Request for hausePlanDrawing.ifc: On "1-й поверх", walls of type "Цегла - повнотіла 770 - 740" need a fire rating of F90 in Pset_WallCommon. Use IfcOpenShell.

First a look at what the model holds.

```python
import ifcopenshell
import ifcopenshell.util.element

model = ifcopenshell.open("hausePlanDrawing.ifc")
print(model.schema)
storey = next(s for s in model.by_type("IfcBuildingStorey") if s.Name == "1-й поверх")
walls = [e for e in ifcopenshell.util.element.get_decomposition(storey) if e.is_a("IfcWall")]
seen = {}
for e in walls:
    element_type = ifcopenshell.util.element.get_type(e)
    key = (element_type.Name if element_type != e and element_type else None, ifcopenshell.util.element.get_pset(e, "Pset_WallCommon", "FireRating"))
    seen[key] = seen.get(key, 0) + 1
for (name, value), count in sorted(seen.items(), key=str):
    print(count, "x", name, "|", value)
```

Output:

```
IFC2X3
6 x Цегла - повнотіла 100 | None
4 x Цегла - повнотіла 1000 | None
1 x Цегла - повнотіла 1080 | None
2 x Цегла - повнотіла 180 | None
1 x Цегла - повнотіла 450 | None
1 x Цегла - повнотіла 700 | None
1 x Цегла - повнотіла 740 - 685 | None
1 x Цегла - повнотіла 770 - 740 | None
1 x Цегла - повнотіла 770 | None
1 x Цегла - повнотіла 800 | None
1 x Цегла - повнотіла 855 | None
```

```python
import ifcopenshell
import ifcopenshell.api.pset
import ifcopenshell.util.element

model = ifcopenshell.open("hausePlanDrawing.ifc")

storey = next(s for s in model.by_type("IfcBuildingStorey") if s.Name == "1-й поверх")
walls = [e for e in ifcopenshell.util.element.get_decomposition(storey) if e.is_a("IfcWall")]

count = 0
for e in walls:
    element_type = ifcopenshell.util.element.get_type(e)
    if element_type in (None, e) or element_type.Name != "Цегла - повнотіла 770 - 740":
        continue
    # add_pset returns the element's existing set when there is one.
    pset = ifcopenshell.api.pset.add_pset(model, product=e, name="Pset_WallCommon")
    ifcopenshell.api.pset.edit_pset(model, pset=pset, properties={"FireRating": "F90"})
    count += 1

print(count, "walls updated")

model.write("hausePlanDrawing_updated.ifc")
```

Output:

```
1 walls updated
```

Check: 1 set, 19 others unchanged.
